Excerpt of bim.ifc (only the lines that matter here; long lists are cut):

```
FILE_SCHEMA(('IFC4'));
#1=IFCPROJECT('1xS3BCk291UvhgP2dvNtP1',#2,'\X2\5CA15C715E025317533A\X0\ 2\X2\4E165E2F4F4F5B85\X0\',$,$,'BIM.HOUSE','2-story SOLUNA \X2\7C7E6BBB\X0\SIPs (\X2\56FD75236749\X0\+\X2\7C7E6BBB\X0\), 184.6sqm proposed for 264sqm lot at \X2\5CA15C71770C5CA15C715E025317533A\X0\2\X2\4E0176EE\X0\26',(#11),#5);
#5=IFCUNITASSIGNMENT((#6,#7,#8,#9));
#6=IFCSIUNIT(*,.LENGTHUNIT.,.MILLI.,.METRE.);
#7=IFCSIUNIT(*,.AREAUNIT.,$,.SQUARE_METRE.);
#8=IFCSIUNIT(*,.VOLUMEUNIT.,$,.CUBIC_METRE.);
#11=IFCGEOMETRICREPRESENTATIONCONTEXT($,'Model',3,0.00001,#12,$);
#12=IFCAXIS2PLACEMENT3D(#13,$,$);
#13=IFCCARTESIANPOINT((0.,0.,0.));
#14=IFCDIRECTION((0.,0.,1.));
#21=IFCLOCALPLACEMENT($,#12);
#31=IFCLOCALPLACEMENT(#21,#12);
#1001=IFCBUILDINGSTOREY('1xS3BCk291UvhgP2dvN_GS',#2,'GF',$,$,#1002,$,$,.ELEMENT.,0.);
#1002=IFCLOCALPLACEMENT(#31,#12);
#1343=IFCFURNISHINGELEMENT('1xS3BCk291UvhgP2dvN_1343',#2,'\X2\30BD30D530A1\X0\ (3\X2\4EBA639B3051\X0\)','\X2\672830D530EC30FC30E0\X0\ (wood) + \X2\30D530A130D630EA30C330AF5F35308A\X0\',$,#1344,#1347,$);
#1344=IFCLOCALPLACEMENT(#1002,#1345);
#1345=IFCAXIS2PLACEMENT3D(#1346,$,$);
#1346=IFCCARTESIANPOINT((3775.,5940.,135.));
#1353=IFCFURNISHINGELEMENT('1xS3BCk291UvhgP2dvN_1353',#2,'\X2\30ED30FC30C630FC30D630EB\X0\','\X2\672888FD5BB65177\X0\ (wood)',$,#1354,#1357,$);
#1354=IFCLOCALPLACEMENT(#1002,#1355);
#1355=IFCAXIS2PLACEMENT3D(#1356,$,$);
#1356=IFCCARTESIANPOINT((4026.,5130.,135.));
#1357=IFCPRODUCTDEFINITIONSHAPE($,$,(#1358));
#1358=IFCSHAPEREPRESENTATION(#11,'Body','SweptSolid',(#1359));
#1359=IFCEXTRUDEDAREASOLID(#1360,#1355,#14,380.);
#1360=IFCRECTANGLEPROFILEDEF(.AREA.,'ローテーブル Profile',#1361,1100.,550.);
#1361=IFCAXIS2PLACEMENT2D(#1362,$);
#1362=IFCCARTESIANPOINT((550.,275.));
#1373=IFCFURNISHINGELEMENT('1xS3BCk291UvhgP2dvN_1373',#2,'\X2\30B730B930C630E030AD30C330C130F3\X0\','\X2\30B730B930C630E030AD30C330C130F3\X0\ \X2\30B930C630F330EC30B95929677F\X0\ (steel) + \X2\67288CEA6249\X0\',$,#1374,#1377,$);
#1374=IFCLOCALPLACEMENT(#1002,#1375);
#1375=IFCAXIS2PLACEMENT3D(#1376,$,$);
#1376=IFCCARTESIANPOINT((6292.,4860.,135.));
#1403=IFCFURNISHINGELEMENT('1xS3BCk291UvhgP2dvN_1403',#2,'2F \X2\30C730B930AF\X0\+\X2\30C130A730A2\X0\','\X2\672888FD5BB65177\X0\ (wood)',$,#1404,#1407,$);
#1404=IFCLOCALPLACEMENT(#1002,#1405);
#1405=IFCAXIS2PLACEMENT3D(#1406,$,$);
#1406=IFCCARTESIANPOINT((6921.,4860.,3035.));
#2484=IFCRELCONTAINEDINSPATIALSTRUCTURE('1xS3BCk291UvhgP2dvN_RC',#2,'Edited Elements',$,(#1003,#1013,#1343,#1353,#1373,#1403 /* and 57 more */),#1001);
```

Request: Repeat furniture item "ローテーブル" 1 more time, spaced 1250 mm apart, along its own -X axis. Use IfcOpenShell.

```python
import ifcopenshell
import ifcopenshell.api.geometry
import ifcopenshell.api.root
import ifcopenshell.util.element
import ifcopenshell.util.placement
import ifcopenshell.util.unit

model = ifcopenshell.open("bim.ifc")
unit_scale = ifcopenshell.util.unit.calculate_unit_scale(model)


def reuse_history(source, copy):
    """copy_class also copies each property set's owner history, people and application; keep the originals."""
    for rel in copy.IsDefinedBy:
        if rel.is_a("IfcRelDefinesByProperties") and (history := rel.RelatingPropertyDefinition.OwnerHistory):
            rel.RelatingPropertyDefinition.OwnerHistory = source.OwnerHistory
            ifcopenshell.util.element.remove_deep2(model, history)


source = model.by_guid("1xS3BCk291UvhgP2dvN_1353")
base = ifcopenshell.util.placement.get_local_placement(source.ObjectPlacement)
step = -base[:3, 0] * 1.25 / unit_scale

for i in range(1, 2):
    copy = ifcopenshell.api.root.copy_class(model, product=source)
    copy.Representation = ifcopenshell.util.element.copy_deep(
        model, source.Representation, exclude=["IfcGeometricRepresentationContext", "IfcRepresentationMap"]
    )
    reuse_history(source, copy)
    matrix = base.copy()
    matrix[:3, 3] += i * step
    print("added at", matrix[:3, 3].round(3) + 0.0)
    ifcopenshell.api.geometry.edit_object_placement(model, product=copy, matrix=matrix, is_si=False)

model.write("bim-out.ifc")
```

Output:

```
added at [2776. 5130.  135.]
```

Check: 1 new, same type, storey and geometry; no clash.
